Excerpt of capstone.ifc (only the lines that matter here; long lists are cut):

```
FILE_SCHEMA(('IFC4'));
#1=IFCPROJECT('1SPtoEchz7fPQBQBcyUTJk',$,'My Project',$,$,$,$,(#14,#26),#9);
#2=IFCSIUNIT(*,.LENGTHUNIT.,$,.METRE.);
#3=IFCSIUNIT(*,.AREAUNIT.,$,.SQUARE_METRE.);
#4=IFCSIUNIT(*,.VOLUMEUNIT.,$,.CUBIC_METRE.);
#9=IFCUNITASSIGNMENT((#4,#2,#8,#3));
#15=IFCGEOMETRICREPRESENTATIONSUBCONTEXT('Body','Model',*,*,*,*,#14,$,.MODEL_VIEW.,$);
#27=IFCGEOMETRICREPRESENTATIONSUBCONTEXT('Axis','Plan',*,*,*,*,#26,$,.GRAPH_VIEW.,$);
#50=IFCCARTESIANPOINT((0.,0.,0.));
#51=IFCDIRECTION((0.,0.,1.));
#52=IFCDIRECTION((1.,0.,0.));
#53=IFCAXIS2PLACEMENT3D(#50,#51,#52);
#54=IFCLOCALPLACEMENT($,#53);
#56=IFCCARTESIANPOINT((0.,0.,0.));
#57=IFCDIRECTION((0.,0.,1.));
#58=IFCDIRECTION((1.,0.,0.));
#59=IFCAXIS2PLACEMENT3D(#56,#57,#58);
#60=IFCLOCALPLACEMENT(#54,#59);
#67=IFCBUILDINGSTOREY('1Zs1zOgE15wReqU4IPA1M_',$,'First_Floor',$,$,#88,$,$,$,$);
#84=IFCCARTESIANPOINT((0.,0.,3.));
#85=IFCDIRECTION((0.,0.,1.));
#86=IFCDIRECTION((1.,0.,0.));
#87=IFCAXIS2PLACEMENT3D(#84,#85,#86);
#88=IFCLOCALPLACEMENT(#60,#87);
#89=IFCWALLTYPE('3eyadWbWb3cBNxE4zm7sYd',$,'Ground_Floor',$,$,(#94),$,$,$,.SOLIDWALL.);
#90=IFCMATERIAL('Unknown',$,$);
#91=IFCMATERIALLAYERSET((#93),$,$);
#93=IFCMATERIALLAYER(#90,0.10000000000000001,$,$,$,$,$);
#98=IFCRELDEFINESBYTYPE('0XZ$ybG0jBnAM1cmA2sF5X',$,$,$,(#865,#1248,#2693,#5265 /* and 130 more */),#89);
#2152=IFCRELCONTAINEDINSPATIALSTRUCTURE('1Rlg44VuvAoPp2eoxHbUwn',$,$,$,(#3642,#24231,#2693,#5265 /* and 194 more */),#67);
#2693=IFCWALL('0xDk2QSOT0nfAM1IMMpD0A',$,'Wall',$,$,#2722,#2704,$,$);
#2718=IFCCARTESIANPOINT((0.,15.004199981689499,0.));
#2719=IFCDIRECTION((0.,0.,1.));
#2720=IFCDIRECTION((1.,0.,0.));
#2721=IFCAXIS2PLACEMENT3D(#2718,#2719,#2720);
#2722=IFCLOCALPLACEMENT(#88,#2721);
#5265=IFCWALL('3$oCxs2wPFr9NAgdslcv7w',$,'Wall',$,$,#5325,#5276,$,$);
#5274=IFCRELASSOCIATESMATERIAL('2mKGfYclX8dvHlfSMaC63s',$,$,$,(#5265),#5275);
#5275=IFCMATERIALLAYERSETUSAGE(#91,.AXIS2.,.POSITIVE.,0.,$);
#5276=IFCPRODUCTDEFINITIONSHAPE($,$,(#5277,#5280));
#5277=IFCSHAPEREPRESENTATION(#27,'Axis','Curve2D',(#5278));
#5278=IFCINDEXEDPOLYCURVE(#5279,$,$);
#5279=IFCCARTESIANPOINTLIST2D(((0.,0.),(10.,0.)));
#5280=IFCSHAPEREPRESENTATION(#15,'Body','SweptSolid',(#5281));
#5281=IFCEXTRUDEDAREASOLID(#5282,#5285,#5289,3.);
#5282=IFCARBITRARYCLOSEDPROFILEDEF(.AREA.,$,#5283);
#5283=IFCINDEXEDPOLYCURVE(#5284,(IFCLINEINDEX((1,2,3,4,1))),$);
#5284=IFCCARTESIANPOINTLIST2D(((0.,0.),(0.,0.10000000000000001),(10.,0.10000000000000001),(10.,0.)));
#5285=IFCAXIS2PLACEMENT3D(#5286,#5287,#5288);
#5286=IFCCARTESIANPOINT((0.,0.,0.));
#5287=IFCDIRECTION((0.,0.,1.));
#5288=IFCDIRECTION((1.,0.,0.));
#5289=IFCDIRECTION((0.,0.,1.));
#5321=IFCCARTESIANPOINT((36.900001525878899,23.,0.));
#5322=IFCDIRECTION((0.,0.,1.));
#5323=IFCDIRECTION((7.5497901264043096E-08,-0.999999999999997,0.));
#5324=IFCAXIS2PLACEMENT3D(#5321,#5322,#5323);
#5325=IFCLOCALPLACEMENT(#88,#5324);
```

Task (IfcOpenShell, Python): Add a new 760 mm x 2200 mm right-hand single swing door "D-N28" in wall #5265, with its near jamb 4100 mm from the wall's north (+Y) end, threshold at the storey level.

```python
import numpy as np
import ifcopenshell
import ifcopenshell.api.feature
import ifcopenshell.api.geometry
import ifcopenshell.api.root
import ifcopenshell.api.spatial
import ifcopenshell.geom
import ifcopenshell.util.element
import ifcopenshell.util.placement
import ifcopenshell.util.representation
import ifcopenshell.util.shape
import ifcopenshell.util.unit

model = ifcopenshell.open("capstone.ifc")
unit_scale = ifcopenshell.util.unit.calculate_unit_scale(model)
settings = ifcopenshell.geom.settings()


def volume(element):
    """Net volume in cubic metres, openings subtracted."""
    shape = ifcopenshell.geom.create_shape(settings, element)
    return ifcopenshell.util.shape.get_volume(shape.geometry)


wall = model.by_id(5265)
storey = ifcopenshell.util.element.get_container(wall, ifc_class="IfcBuildingStorey")
context = ifcopenshell.util.representation.get_context(model, "Model", "Body", "MODEL_VIEW")
before = volume(wall)

width, height, from_end, sill = 0.76, 2.2, 4.1, 0.0  # metres

# The wall runs along its own X axis, and the end named is its -X end.
wall_shape = ifcopenshell.geom.create_shape(settings, wall)
x, y, z = ifcopenshell.util.shape.get_vertices(wall_shape.geometry).T
start = x.min() + from_end
face, thickness = float(y.min()), float(y.max() - y.min())
wall_matrix = ifcopenshell.util.placement.get_local_placement(wall.ObjectPlacement)
level = ifcopenshell.util.placement.get_local_placement(storey.ObjectPlacement)[2, 3]


def in_wall(x, y):
    """Placement at x, y metres in the wall's axes, at sill height."""
    matrix = wall_matrix.copy()
    matrix[:, 3] = wall_matrix @ np.array([x / unit_scale, y / unit_scale, 0.0, 1.0])
    matrix[2, 3] = level + sill / unit_scale
    return matrix


# Opening: a box that overshoots both wall faces by 50 mm.
opening = ifcopenshell.api.root.create_entity(model, ifc_class="IfcOpeningElement", predefined_type="OPENING")
box = ifcopenshell.api.geometry.add_wall_representation(
    model, context=context, length=width, height=height, thickness=thickness + 0.1
)
ifcopenshell.api.geometry.assign_representation(model, product=opening, representation=box)
ifcopenshell.api.geometry.edit_object_placement(model, product=opening, matrix=in_wall(start, face - 0.05), is_si=False)
ifcopenshell.api.feature.add_feature(model, feature=opening, element=wall)

door = ifcopenshell.api.root.create_entity(model, ifc_class="IfcDoor", name="D-N28", predefined_type="DOOR")
door.OverallWidth, door.OverallHeight = width / unit_scale, height / unit_scale
door.OperationType = "SINGLE_SWING_RIGHT"
body = ifcopenshell.api.geometry.add_door_representation(
    model,
    context=context,
    overall_width=door.OverallWidth,
    overall_height=door.OverallHeight,
    operation_type="SINGLE_SWING_RIGHT",
    lining_properties={"LiningDepth": thickness / unit_scale, "ThresholdDepth": thickness / unit_scale},
)
ifcopenshell.api.geometry.assign_representation(model, product=door, representation=body)
ifcopenshell.api.spatial.assign_container(model, products=[door], relating_structure=storey)
ifcopenshell.api.feature.add_filling(model, opening=opening, element=door)

# The lining spans the wall, so the door starts at the wall face.
ifcopenshell.api.geometry.edit_object_placement(model, product=door, matrix=in_wall(start, face), is_si=False)

after = volume(wall)

print(f"wall volume {before:.3f} -> {after:.3f} m3")

model.write("capstone_edited.ifc")
```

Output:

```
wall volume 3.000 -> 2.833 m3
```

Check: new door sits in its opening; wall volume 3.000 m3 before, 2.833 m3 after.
